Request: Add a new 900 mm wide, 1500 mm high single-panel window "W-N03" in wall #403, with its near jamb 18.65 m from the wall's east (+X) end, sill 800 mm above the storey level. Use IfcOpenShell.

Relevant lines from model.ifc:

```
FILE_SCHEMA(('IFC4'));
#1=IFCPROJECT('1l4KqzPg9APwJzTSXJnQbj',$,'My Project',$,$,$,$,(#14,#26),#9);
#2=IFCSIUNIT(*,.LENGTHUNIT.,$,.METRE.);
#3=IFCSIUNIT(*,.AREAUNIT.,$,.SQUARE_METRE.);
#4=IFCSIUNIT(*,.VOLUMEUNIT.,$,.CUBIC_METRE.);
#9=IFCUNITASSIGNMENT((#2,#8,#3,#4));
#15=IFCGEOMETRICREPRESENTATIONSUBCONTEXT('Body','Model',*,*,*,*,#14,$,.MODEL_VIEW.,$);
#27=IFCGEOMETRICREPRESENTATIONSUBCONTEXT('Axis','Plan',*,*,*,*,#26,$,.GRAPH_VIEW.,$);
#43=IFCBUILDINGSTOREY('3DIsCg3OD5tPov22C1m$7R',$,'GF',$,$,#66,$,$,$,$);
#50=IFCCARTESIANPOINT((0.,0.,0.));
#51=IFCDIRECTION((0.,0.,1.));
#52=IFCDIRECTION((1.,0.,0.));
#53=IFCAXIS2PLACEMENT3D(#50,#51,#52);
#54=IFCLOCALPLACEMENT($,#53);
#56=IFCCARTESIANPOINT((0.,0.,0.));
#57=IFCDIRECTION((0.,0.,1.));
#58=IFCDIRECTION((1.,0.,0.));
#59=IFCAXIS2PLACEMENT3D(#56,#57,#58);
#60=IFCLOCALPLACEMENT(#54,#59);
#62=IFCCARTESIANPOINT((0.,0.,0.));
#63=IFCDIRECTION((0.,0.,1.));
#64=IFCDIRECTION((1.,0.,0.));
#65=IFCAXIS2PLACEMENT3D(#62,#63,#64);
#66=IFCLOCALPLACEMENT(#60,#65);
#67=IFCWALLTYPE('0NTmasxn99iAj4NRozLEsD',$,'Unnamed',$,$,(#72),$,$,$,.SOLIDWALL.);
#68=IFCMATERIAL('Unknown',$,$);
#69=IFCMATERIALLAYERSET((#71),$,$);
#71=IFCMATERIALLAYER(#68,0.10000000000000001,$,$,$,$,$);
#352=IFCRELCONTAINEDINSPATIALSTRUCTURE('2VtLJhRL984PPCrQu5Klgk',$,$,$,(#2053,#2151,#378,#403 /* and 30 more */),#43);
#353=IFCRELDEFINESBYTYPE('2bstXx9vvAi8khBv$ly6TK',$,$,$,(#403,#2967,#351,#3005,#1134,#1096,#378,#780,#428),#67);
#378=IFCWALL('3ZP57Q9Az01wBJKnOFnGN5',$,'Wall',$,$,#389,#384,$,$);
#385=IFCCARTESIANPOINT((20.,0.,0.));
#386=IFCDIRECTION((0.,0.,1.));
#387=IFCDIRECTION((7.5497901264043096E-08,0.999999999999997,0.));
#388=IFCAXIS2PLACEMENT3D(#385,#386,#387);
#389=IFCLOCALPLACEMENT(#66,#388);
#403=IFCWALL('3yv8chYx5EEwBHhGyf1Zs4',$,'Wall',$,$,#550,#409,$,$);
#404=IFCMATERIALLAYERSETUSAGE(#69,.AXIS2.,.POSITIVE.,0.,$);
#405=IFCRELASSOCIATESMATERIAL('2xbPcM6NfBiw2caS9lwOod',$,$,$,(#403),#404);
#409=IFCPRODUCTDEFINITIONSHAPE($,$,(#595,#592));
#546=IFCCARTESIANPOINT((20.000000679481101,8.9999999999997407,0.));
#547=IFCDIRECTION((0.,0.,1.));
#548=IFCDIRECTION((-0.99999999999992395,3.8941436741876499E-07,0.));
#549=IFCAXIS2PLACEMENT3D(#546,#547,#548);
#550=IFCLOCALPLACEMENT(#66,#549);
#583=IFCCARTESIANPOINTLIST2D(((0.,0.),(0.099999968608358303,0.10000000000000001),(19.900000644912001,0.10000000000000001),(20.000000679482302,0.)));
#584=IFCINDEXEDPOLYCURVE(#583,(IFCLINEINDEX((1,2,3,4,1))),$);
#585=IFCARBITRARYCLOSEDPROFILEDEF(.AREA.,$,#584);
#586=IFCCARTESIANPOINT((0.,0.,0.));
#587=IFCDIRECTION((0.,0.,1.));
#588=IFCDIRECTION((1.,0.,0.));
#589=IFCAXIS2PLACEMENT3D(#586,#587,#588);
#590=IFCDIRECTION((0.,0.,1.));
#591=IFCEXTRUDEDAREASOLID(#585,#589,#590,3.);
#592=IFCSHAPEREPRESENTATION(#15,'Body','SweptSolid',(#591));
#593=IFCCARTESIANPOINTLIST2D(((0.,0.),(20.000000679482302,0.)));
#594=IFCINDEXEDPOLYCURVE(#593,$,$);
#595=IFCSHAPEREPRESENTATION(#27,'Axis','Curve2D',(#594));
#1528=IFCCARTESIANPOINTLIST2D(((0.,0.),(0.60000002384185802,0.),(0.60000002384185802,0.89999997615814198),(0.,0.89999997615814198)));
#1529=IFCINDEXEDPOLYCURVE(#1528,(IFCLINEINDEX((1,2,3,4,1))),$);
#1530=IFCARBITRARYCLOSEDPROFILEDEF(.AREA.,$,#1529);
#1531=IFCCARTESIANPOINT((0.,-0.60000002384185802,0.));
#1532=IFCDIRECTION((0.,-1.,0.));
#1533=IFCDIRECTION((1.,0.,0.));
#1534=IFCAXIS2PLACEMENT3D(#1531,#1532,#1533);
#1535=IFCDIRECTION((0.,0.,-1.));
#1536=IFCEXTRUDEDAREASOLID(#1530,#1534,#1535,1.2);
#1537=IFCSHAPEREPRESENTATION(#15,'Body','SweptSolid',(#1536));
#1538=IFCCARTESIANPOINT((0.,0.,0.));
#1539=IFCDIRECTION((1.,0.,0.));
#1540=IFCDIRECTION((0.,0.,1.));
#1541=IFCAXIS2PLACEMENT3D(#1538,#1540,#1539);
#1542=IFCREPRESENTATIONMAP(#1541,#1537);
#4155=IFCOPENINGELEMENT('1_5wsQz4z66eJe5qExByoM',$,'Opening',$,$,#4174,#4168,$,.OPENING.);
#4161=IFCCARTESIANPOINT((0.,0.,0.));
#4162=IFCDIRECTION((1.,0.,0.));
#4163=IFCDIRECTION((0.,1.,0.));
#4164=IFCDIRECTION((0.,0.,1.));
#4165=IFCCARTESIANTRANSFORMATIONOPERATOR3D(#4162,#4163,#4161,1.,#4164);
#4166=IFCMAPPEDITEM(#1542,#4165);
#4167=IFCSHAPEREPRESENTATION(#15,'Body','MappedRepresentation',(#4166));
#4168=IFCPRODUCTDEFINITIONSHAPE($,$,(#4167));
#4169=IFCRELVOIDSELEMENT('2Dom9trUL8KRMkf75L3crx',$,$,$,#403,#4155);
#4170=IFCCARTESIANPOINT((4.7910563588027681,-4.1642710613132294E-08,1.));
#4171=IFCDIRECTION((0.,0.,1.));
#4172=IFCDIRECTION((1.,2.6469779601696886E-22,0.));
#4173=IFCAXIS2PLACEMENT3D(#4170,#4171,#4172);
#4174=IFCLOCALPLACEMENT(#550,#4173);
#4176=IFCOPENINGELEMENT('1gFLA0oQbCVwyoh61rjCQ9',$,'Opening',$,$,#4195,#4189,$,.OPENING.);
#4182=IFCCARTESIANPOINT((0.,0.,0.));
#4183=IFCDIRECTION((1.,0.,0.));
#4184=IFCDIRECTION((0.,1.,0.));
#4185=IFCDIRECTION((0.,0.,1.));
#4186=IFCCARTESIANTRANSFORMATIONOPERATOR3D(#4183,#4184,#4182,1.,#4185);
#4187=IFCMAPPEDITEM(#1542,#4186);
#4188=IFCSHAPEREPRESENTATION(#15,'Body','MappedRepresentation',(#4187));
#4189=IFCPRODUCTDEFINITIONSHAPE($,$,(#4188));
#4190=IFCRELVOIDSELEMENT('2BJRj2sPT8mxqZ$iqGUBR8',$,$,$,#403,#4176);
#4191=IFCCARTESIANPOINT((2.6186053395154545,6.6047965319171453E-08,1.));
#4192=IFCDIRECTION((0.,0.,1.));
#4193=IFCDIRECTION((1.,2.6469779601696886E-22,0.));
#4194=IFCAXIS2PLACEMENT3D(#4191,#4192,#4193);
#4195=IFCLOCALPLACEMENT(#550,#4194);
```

```python
import numpy as np
import ifcopenshell
import ifcopenshell.api.feature
import ifcopenshell.api.geometry
import ifcopenshell.api.root
import ifcopenshell.api.spatial
import ifcopenshell.geom
import ifcopenshell.util.element
import ifcopenshell.util.placement
import ifcopenshell.util.representation
import ifcopenshell.util.shape
import ifcopenshell.util.unit

model = ifcopenshell.open("model.ifc")
unit_scale = ifcopenshell.util.unit.calculate_unit_scale(model)
settings = ifcopenshell.geom.settings()


def volume(element):
    """Net volume in cubic metres, openings subtracted."""
    shape = ifcopenshell.geom.create_shape(settings, element)
    return ifcopenshell.util.shape.get_volume(shape.geometry)


wall = model.by_guid("3yv8chYx5EEwBHhGyf1Zs4")
storey = ifcopenshell.util.element.get_container(wall, ifc_class="IfcBuildingStorey")
context = ifcopenshell.util.representation.get_context(model, "Model", "Body", "MODEL_VIEW")
before = volume(wall)

width, height, from_end, sill = 0.9, 1.5, 18.65, 0.8  # metres

# The wall runs along its own X axis, and the end named is its -X end.
wall_shape = ifcopenshell.geom.create_shape(settings, wall)
x, y, z = ifcopenshell.util.shape.get_vertices(wall_shape.geometry).T
start = x.min() + from_end
face, thickness = float(y.min()), float(y.max() - y.min())
wall_matrix = ifcopenshell.util.placement.get_local_placement(wall.ObjectPlacement)
level = ifcopenshell.util.placement.get_local_placement(storey.ObjectPlacement)[2, 3]


def in_wall(x, y):
    """Placement at x, y metres in the wall's axes, at sill height."""
    matrix = wall_matrix.copy()
    matrix[:, 3] = wall_matrix @ np.array([x / unit_scale, y / unit_scale, 0.0, 1.0])
    matrix[2, 3] = level + sill / unit_scale
    return matrix


# Opening: a box that overshoots both wall faces by 50 mm.
opening = ifcopenshell.api.root.create_entity(model, ifc_class="IfcOpeningElement", predefined_type="OPENING")
box = ifcopenshell.api.geometry.add_wall_representation(
    model, context=context, length=width, height=height, thickness=thickness + 0.1
)
ifcopenshell.api.geometry.assign_representation(model, product=opening, representation=box)
ifcopenshell.api.geometry.edit_object_placement(model, product=opening, matrix=in_wall(start, face - 0.05), is_si=False)
ifcopenshell.api.feature.add_feature(model, feature=opening, element=wall)

window = ifcopenshell.api.root.create_entity(model, ifc_class="IfcWindow", name="W-N03", predefined_type="WINDOW")
window.OverallWidth, window.OverallHeight = width / unit_scale, height / unit_scale
window.PartitioningType = "SINGLE_PANEL"
body = ifcopenshell.api.geometry.add_window_representation(
    model,
    context=context,
    overall_width=window.OverallWidth,
    overall_height=window.OverallHeight,
    partition_type="SINGLE_PANEL",
)
ifcopenshell.api.geometry.assign_representation(model, product=window, representation=body)
ifcopenshell.api.spatial.assign_container(model, products=[window], relating_structure=storey)
ifcopenshell.api.feature.add_filling(model, opening=opening, element=window)

# Centre the window in the wall's thickness.
ifcopenshell.api.geometry.edit_object_placement(model, product=window, matrix=in_wall(start, face), is_si=False)
window_shape = ifcopenshell.geom.create_shape(settings, window)
depth = ifcopenshell.util.shape.get_vertices(window_shape.geometry)[:, 1]
offset = face + thickness / 2 - (depth.min() + depth.max()) / 2
ifcopenshell.api.geometry.edit_object_placement(model, product=window, matrix=in_wall(start, offset), is_si=False)

after = volume(wall)

print(f"wall volume {before:.3f} -> {after:.3f} m3")

model.write("model_rev.ifc")
```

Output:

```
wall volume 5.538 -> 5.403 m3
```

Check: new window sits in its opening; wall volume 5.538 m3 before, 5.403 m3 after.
